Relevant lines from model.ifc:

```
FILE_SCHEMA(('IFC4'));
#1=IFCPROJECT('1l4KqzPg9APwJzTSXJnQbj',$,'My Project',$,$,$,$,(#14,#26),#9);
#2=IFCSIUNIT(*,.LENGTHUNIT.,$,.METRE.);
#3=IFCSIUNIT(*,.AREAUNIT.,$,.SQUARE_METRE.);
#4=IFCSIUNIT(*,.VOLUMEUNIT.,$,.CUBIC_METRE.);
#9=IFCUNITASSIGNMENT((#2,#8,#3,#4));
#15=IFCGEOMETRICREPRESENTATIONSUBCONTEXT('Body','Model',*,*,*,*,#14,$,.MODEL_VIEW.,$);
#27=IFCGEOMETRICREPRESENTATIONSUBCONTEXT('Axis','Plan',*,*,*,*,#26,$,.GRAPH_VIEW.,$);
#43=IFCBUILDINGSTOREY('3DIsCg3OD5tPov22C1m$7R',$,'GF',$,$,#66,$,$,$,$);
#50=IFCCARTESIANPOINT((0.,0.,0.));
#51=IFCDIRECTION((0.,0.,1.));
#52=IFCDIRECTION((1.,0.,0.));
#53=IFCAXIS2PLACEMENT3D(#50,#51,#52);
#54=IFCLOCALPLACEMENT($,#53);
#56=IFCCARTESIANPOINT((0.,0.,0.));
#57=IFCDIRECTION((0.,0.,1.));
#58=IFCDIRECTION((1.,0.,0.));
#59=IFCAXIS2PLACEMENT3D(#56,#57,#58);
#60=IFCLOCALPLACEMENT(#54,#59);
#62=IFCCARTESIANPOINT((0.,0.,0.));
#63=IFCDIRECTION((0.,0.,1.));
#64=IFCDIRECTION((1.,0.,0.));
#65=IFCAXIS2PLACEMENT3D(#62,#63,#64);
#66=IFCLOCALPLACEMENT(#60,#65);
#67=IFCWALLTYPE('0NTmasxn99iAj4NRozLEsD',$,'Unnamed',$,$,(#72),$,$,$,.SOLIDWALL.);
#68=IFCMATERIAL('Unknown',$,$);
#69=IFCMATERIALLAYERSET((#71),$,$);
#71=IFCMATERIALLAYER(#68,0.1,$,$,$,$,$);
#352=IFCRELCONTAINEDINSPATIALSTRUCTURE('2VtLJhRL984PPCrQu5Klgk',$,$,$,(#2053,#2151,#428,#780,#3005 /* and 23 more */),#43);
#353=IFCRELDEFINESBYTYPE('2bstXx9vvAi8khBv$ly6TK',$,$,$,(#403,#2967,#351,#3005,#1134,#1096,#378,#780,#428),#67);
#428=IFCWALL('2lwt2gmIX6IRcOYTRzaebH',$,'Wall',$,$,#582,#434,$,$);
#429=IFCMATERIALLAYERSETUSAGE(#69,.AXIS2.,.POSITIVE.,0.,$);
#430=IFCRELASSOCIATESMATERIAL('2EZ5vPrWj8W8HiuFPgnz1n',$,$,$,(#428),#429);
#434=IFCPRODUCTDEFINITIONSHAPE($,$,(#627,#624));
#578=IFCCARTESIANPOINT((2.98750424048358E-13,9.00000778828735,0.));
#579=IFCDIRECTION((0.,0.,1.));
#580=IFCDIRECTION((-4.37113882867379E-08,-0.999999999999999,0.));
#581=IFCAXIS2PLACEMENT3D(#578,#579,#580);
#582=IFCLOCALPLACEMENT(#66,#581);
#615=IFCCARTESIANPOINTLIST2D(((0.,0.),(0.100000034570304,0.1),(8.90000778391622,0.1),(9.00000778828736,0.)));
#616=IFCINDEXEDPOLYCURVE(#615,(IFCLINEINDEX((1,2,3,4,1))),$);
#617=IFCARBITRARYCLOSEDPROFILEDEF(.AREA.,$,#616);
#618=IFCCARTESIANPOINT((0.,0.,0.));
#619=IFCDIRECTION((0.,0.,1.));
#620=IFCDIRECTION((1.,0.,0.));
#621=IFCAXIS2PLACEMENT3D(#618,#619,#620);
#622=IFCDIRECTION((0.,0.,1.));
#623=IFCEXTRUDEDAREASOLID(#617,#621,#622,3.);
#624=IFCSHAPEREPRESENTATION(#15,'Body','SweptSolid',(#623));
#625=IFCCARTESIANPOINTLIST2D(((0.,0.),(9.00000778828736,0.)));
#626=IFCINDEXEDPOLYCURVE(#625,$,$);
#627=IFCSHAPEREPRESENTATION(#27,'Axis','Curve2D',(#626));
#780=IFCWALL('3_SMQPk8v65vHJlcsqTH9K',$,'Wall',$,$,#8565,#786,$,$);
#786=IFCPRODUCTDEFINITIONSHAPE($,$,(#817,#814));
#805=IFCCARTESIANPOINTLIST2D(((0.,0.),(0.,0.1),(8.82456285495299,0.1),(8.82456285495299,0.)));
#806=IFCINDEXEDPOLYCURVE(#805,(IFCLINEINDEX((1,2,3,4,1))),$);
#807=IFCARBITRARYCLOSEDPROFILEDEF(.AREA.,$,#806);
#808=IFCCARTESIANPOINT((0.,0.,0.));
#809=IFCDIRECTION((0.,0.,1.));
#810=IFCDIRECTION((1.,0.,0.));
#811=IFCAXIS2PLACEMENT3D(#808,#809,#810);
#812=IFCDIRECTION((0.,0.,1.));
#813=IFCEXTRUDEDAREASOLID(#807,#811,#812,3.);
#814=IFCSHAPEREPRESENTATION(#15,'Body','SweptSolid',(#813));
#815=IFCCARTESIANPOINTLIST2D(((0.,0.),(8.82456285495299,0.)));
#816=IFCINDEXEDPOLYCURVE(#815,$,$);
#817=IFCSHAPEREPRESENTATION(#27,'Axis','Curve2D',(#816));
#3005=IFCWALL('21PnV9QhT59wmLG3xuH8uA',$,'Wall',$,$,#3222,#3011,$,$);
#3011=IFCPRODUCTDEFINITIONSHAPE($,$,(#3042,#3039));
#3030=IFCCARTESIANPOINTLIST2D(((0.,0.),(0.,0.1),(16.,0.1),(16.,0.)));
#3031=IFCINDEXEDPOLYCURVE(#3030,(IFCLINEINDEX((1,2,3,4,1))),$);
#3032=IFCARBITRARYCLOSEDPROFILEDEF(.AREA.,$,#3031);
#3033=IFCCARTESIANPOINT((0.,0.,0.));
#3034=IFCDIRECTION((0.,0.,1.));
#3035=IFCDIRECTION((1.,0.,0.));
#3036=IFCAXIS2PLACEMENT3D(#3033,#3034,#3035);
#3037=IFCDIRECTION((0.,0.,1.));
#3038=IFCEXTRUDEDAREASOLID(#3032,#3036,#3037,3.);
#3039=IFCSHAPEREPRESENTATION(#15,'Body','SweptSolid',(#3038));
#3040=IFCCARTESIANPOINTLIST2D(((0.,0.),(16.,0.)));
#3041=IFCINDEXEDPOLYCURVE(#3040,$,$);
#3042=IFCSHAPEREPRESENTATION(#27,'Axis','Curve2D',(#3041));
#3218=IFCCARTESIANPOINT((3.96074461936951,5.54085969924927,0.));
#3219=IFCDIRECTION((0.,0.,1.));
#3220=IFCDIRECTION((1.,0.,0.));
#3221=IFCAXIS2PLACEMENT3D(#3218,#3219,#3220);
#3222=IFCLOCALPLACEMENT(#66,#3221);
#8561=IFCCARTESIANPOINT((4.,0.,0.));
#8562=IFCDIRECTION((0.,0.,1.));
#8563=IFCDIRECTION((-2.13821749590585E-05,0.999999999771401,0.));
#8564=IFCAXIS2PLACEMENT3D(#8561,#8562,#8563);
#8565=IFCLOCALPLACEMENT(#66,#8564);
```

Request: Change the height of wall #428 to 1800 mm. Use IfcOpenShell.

```python
import ifcopenshell
import ifcopenshell.geom
import ifcopenshell.util.representation
import ifcopenshell.util.shape

model = ifcopenshell.open("model.ifc")
settings = ifcopenshell.geom.settings()


def volume(element):
    """Net volume in cubic metres, openings subtracted."""
    shape = ifcopenshell.geom.create_shape(settings, element)
    return ifcopenshell.util.shape.get_volume(shape.geometry)


wall = model.by_guid("2lwt2gmIX6IRcOYTRzaebH")
before = volume(wall)

body = ifcopenshell.util.representation.get_representation(wall, "Model", "Body")
solid = body.Items[0]
old_height = solid.Depth
solid.Depth = 1.8
after = volume(wall)

print(f"height {old_height:g} -> {solid.Depth:g}, volume {before:.3f} -> {after:.3f} m3")

model.write("model_updated.ifc")
```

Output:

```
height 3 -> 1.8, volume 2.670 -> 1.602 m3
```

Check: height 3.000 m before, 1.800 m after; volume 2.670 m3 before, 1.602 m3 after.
